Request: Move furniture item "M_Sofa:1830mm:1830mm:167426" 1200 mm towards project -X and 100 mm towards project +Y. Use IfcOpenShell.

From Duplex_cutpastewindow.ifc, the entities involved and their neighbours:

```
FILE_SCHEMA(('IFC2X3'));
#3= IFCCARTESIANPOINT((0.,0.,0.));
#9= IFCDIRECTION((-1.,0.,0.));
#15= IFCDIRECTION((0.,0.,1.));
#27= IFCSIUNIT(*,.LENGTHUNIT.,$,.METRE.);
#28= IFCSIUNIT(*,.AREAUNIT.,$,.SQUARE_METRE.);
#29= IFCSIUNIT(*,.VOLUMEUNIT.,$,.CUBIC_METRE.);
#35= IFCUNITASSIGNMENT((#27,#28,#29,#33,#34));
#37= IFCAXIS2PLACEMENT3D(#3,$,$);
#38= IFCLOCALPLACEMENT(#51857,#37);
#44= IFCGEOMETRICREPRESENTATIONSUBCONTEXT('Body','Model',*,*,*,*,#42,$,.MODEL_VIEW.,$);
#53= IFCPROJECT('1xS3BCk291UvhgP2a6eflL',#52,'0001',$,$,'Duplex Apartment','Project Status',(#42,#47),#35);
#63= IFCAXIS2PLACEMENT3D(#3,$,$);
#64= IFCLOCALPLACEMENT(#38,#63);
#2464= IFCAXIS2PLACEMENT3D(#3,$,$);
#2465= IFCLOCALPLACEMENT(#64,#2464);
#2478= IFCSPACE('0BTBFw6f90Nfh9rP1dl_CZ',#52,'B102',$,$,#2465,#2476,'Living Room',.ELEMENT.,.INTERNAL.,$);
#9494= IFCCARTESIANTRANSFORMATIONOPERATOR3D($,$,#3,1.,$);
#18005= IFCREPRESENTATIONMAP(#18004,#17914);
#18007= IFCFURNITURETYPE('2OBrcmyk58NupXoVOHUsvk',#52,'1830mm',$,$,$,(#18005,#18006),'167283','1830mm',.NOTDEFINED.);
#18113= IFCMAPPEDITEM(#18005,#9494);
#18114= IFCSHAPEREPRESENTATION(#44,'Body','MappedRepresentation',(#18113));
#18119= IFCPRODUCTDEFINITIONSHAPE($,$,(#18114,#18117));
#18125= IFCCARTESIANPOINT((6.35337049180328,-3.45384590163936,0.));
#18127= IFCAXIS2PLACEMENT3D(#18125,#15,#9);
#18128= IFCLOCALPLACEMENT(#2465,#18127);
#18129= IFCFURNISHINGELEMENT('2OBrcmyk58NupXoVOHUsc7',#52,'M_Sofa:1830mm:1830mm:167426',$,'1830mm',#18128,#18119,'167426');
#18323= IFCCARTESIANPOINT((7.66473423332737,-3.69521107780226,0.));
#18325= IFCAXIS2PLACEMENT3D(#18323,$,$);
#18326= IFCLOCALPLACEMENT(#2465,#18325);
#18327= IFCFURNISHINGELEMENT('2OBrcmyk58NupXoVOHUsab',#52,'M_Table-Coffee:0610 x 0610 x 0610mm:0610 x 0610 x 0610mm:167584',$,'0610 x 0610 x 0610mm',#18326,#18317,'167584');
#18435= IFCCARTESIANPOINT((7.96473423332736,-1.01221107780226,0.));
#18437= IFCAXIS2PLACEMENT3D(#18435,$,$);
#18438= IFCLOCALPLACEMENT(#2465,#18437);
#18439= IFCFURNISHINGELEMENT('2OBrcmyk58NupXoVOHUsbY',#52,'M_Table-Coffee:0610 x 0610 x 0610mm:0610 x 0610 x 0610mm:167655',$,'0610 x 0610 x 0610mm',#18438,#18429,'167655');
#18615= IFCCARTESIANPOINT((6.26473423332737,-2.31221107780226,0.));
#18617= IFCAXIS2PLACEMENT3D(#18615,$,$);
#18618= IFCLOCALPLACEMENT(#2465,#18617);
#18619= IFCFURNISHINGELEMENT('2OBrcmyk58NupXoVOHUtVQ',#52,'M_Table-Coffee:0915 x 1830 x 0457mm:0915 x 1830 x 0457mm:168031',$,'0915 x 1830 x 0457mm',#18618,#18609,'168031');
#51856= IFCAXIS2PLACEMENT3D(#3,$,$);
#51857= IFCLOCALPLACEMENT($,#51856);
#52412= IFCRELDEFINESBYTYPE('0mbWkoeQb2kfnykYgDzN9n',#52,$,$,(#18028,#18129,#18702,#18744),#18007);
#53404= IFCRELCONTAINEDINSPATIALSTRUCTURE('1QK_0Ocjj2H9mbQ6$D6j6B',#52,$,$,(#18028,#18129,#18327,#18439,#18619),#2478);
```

```python
import ifcopenshell
import ifcopenshell.api.geometry
import ifcopenshell.util.placement
import ifcopenshell.util.unit

model = ifcopenshell.open("Duplex_cutpastewindow.ifc")
unit_scale = ifcopenshell.util.unit.calculate_unit_scale(model)

item = model.by_guid("2OBrcmyk58NupXoVOHUsc7")
matrix = ifcopenshell.util.placement.get_local_placement(item.ObjectPlacement)
matrix[0, 3] -= 1.2 / unit_scale
matrix[1, 3] += 0.1 / unit_scale
ifcopenshell.api.geometry.edit_object_placement(model, product=item, matrix=matrix, is_si=False)

print(ifcopenshell.util.placement.get_local_placement(item.ObjectPlacement).round(3) + 0.0)

model.write("Duplex_cutpastewindow_rev.ifc")
```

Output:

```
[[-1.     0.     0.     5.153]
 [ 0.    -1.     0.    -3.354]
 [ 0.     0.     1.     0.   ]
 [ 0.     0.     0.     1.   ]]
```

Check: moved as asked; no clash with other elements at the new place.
